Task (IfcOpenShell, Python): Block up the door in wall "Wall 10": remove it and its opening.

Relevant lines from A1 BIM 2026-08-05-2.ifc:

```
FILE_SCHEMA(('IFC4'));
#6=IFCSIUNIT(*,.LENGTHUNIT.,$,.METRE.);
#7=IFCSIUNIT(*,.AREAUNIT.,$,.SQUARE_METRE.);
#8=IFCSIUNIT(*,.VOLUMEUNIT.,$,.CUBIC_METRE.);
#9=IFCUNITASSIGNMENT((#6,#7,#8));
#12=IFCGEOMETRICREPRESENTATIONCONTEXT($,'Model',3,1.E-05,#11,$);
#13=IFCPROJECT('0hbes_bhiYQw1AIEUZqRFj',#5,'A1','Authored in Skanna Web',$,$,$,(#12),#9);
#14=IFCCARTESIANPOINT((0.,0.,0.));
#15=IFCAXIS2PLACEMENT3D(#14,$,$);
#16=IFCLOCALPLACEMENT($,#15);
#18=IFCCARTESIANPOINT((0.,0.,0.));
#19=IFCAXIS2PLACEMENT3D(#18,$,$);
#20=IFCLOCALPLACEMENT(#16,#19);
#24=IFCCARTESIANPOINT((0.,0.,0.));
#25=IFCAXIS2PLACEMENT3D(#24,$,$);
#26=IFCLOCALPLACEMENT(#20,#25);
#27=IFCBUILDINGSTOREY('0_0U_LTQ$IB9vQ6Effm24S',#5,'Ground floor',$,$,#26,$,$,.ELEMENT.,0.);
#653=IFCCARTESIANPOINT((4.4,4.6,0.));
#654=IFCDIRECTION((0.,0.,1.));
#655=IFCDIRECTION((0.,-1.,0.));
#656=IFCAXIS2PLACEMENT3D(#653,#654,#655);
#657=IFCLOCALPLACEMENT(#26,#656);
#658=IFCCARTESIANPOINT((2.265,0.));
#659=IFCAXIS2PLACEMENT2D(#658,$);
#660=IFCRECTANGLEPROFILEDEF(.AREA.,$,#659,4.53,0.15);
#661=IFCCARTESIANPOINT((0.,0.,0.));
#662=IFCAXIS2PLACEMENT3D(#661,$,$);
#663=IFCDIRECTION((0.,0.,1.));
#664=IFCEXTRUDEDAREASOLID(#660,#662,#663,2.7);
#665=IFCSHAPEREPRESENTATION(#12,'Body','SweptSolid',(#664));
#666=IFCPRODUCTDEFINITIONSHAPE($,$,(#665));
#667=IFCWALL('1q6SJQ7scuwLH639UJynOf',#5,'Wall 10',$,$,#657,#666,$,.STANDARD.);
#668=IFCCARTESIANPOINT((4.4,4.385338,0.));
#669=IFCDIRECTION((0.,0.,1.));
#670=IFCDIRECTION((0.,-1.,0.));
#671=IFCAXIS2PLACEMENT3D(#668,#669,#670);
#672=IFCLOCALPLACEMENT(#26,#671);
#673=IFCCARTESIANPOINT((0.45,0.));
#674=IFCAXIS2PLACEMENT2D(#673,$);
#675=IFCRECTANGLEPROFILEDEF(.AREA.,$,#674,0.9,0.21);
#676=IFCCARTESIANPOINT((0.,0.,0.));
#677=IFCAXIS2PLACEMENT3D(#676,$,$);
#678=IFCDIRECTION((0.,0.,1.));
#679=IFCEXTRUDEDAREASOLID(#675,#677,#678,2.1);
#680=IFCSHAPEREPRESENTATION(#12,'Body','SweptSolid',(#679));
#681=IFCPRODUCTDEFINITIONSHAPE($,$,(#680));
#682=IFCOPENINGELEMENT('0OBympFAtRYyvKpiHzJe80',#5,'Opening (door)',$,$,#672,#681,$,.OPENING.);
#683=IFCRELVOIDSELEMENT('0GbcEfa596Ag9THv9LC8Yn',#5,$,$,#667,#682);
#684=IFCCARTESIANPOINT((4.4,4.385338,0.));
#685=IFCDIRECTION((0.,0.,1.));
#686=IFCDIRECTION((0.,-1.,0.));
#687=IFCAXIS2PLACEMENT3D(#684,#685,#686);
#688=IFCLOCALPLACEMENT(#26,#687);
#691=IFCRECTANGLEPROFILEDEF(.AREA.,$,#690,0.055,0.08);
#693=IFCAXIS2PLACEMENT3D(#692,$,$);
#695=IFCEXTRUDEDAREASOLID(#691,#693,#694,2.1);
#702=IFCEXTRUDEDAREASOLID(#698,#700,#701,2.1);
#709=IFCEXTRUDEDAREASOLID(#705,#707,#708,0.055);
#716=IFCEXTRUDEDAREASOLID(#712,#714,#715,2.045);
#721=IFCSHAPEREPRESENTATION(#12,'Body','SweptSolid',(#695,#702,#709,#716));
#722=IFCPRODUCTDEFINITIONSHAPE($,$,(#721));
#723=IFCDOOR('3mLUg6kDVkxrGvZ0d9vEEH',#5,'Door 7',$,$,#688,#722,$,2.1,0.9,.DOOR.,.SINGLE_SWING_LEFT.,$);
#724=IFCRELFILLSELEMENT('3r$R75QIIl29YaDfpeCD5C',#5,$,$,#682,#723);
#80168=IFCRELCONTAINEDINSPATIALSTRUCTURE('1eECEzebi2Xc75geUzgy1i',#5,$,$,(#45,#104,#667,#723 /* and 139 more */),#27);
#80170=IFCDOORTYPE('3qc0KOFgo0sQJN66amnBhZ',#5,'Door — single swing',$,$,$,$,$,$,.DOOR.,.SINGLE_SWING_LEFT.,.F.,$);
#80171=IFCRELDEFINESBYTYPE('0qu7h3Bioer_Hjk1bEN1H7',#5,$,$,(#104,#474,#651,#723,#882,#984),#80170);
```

```python
import ifcopenshell
import ifcopenshell.api.feature
import ifcopenshell.api.root
import ifcopenshell.geom
import ifcopenshell.util.shape

model = ifcopenshell.open("A1 BIM 2026-08-05-2.ifc")
settings = ifcopenshell.geom.settings()


def volume(element):
    """Net volume in cubic metres, openings subtracted."""
    shape = ifcopenshell.geom.create_shape(settings, element)
    return ifcopenshell.util.shape.get_volume(shape.geometry)


door = model.by_guid("3mLUg6kDVkxrGvZ0d9vEEH")
opening = door.FillsVoids[0].RelatingOpeningElement
wall = opening.VoidsElements[0].RelatingBuildingElement
before = volume(wall)

ifcopenshell.api.root.remove_product(model, product=door)
ifcopenshell.api.feature.remove_feature(model, feature=opening)

after = volume(wall)

print(f"wall volume {before:.3f} -> {after:.3f} m3")

model.write("A1 BIM 2026-08-05-2_edited.ifc")
```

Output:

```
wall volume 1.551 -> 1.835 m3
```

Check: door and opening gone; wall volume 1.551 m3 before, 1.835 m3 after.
